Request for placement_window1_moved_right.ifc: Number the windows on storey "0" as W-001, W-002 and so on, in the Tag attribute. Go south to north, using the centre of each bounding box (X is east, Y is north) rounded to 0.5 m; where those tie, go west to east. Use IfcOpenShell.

First a look at what the model holds.

```python
import ifcopenshell
import ifcopenshell.util.element
import ifcopenshell.util.placement

model = ifcopenshell.open("placement_window1_moved_right.ifc")
print(model.schema)
storey = next(s for s in model.by_type("IfcBuildingStorey") if s.Name == "0")
windows = [e for e in ifcopenshell.util.element.get_decomposition(storey) if e.is_a("IfcWindow")]
for e in sorted(windows, key=lambda e: e.id()):
    origin = ifcopenshell.util.placement.get_local_placement(e.ObjectPlacement)[:3, 3]
    print(e.id(), e.Tag, e.Name, origin.round(2) + 0.0, sep=" | ")
```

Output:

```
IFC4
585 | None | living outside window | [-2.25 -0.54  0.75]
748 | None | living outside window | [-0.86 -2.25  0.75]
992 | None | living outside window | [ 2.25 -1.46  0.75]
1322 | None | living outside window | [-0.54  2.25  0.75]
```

```python
import ifcopenshell
import ifcopenshell.geom
import ifcopenshell.util.element
import ifcopenshell.util.shape

model = ifcopenshell.open("placement_window1_moved_right.ifc")
settings = ifcopenshell.geom.settings()
settings.set("use-world-coords", True)


def centre(element):
    shape = ifcopenshell.geom.create_shape(settings, element)
    return ifcopenshell.util.shape.get_bbox_centroid(shape.geometry)


storey = next(s for s in model.by_type("IfcBuildingStorey") if s.Name == "0")
windows = [e for e in ifcopenshell.util.element.get_decomposition(storey) if e.is_a("IfcWindow")]

# Insertion points can sit at a corner or the storey origin, so sort by the geometry (in metres).
centres = {e: centre(e) for e in windows}
windows.sort(key=lambda e: (round(centres[e][1] / 0.5), centres[e][0]))

for i, e in enumerate(windows, start=1):
    number = f"W-0{i:02d}"
    e.Tag = number
    print(e.id(), number)

model.write("placement_window1_moved_right_updated.ifc")
```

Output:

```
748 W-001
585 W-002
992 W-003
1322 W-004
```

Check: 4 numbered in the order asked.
